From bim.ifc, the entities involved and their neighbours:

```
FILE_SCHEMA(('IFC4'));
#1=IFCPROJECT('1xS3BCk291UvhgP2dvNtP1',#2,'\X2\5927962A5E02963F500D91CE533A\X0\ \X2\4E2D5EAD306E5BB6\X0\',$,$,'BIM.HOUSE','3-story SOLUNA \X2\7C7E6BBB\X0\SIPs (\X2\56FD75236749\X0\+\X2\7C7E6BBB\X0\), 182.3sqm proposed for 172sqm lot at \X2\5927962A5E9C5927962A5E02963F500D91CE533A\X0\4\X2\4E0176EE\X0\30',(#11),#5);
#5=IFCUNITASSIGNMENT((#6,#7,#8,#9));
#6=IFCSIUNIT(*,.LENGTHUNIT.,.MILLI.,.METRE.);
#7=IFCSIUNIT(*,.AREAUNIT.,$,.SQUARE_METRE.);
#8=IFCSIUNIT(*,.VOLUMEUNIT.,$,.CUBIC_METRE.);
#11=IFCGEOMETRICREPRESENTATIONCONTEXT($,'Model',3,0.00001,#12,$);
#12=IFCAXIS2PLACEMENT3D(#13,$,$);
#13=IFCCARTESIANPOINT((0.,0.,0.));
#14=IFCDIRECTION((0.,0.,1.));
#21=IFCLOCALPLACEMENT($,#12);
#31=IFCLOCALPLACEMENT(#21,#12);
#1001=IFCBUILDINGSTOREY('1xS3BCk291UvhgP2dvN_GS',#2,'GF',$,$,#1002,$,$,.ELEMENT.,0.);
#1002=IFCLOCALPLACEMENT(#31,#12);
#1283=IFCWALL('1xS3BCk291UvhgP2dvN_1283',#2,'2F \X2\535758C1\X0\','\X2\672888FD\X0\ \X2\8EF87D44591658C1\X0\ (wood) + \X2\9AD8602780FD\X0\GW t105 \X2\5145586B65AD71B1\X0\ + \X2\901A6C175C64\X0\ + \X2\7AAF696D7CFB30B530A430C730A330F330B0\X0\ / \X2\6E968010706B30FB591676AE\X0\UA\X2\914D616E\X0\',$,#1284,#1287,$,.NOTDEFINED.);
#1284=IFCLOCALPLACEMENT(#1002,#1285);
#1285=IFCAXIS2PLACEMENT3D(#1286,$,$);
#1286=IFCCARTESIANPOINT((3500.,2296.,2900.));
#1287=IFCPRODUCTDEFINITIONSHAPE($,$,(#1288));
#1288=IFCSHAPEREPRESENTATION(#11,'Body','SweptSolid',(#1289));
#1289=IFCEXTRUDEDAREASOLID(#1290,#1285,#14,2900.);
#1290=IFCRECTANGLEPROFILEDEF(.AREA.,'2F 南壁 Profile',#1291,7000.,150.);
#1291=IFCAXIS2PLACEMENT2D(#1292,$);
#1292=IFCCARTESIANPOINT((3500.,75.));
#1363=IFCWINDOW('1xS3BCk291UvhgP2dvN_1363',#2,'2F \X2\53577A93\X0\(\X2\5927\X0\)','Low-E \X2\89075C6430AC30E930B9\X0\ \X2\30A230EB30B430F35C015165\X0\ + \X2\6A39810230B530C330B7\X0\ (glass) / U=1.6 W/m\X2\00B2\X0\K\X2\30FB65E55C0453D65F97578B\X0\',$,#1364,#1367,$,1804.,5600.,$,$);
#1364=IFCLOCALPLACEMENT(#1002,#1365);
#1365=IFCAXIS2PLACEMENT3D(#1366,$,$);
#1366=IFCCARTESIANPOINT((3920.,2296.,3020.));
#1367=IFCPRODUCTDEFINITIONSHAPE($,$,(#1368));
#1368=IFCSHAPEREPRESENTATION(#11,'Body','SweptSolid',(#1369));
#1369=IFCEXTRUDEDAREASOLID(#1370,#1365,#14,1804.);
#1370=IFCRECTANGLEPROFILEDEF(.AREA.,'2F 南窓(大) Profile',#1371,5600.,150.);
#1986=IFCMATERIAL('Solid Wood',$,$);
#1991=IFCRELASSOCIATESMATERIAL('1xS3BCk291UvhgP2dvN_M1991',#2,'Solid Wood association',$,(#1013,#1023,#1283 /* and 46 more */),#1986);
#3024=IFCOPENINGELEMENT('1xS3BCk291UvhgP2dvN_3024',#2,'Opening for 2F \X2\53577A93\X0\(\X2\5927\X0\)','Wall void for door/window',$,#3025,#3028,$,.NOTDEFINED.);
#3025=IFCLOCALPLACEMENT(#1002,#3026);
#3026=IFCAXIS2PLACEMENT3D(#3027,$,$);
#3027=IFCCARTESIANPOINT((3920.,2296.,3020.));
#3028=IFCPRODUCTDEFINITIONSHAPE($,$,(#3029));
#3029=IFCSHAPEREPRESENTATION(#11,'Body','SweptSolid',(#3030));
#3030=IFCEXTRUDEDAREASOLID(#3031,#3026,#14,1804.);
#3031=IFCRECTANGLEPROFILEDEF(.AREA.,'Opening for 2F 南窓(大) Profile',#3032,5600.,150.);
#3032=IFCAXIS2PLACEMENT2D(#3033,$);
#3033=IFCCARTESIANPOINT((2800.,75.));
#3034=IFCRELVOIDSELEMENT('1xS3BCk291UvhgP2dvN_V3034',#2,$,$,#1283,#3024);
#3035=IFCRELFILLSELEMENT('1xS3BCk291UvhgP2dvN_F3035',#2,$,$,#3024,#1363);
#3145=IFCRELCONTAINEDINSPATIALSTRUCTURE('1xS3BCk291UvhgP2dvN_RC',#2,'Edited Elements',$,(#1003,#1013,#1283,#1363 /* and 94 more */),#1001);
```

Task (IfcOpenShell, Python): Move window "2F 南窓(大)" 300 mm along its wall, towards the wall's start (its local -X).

```python
import ifcopenshell
import ifcopenshell.api.geometry
import ifcopenshell.util.placement

model = ifcopenshell.open("bim.ifc")

window = model.by_guid("1xS3BCk291UvhgP2dvN_1363")
opening = window.FillsVoids[0].RelatingOpeningElement
wall = opening.VoidsElements[0].RelatingBuildingElement

wall_matrix = ifcopenshell.util.placement.get_local_placement(wall.ObjectPlacement)
shift = wall_matrix[:3, 0] * -300.0
before = ifcopenshell.util.placement.get_local_placement(window.ObjectPlacement)[:3, 3].copy()

# The window is not placed relative to its opening, so move both.
for product in (opening, window):
    matrix = ifcopenshell.util.placement.get_local_placement(product.ObjectPlacement)
    matrix[:3, 3] += shift
    ifcopenshell.api.geometry.edit_object_placement(model, product=product, matrix=matrix, is_si=False)

after = ifcopenshell.util.placement.get_local_placement(window.ObjectPlacement)[:3, 3]
print("window moved by", (after - before).round(3) + 0.0)

model.write("bim_v2.ifc")
```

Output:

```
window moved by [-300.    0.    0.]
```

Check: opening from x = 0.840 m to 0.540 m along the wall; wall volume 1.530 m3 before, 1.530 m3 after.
